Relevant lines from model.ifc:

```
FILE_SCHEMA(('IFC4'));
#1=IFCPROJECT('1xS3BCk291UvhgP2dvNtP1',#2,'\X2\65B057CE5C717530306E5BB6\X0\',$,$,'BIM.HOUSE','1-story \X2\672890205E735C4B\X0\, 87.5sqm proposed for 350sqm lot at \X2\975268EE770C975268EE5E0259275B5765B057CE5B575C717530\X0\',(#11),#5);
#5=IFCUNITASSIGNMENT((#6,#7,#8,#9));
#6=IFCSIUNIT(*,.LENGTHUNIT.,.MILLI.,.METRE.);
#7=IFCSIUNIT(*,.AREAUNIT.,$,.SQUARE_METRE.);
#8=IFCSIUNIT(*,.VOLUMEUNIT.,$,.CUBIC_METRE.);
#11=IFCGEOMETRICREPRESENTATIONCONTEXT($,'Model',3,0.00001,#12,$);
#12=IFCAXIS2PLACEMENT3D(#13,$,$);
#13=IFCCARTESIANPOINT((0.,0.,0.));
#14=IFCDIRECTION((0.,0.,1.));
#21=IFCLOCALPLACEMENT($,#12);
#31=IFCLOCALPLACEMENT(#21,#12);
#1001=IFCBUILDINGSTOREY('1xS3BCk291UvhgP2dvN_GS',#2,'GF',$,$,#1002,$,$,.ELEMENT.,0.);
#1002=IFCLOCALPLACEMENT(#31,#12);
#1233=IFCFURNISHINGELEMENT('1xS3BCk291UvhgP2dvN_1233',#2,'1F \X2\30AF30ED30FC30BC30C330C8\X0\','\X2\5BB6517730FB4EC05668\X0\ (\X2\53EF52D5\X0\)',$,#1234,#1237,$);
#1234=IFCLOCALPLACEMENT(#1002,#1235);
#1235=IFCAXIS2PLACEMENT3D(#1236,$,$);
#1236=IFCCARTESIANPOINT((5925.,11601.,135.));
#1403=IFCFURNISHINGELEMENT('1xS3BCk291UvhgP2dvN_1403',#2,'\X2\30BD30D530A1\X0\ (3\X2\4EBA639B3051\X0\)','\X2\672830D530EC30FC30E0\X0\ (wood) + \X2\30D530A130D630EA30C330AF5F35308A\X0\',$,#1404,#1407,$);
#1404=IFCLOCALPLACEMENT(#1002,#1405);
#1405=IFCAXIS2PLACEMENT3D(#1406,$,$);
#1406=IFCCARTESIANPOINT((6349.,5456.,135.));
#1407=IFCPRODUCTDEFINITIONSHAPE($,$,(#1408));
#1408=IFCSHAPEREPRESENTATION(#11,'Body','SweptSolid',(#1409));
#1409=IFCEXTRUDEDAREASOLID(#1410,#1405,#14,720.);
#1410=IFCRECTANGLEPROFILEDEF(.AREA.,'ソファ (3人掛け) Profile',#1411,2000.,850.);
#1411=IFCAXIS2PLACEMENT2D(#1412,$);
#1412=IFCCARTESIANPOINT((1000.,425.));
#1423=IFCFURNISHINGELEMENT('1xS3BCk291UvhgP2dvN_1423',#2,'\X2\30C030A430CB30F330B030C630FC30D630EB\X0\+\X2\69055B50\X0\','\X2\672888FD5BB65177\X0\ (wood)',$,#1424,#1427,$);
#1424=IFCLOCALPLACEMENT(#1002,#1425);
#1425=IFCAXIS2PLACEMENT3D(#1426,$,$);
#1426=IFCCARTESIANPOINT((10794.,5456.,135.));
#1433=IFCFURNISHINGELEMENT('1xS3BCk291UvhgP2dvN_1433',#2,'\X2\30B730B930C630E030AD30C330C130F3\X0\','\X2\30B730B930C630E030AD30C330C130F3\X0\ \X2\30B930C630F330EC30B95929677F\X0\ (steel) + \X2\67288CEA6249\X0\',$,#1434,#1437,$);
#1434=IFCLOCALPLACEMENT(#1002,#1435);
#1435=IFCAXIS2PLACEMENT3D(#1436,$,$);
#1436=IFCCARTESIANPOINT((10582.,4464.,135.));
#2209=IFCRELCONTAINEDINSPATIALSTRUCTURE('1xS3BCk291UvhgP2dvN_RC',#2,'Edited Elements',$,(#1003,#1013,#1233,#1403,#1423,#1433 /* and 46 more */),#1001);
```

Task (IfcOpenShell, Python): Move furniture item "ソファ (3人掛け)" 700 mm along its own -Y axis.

```python
import ifcopenshell
import ifcopenshell.api.geometry
import ifcopenshell.util.placement
import ifcopenshell.util.unit

model = ifcopenshell.open("model.ifc")
unit_scale = ifcopenshell.util.unit.calculate_unit_scale(model)

item = model.by_id(1403)
matrix = ifcopenshell.util.placement.get_local_placement(item.ObjectPlacement)
matrix[:3, 3] -= matrix[:3, 1] * 0.7 / unit_scale
ifcopenshell.api.geometry.edit_object_placement(model, product=item, matrix=matrix, is_si=False)

print(ifcopenshell.util.placement.get_local_placement(item.ObjectPlacement).round(3) + 0.0)

model.write("model-out.ifc")
```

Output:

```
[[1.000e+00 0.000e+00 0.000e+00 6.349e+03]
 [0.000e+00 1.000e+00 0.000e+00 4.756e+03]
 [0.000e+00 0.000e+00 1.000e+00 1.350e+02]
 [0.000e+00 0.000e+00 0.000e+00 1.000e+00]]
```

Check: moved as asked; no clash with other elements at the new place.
